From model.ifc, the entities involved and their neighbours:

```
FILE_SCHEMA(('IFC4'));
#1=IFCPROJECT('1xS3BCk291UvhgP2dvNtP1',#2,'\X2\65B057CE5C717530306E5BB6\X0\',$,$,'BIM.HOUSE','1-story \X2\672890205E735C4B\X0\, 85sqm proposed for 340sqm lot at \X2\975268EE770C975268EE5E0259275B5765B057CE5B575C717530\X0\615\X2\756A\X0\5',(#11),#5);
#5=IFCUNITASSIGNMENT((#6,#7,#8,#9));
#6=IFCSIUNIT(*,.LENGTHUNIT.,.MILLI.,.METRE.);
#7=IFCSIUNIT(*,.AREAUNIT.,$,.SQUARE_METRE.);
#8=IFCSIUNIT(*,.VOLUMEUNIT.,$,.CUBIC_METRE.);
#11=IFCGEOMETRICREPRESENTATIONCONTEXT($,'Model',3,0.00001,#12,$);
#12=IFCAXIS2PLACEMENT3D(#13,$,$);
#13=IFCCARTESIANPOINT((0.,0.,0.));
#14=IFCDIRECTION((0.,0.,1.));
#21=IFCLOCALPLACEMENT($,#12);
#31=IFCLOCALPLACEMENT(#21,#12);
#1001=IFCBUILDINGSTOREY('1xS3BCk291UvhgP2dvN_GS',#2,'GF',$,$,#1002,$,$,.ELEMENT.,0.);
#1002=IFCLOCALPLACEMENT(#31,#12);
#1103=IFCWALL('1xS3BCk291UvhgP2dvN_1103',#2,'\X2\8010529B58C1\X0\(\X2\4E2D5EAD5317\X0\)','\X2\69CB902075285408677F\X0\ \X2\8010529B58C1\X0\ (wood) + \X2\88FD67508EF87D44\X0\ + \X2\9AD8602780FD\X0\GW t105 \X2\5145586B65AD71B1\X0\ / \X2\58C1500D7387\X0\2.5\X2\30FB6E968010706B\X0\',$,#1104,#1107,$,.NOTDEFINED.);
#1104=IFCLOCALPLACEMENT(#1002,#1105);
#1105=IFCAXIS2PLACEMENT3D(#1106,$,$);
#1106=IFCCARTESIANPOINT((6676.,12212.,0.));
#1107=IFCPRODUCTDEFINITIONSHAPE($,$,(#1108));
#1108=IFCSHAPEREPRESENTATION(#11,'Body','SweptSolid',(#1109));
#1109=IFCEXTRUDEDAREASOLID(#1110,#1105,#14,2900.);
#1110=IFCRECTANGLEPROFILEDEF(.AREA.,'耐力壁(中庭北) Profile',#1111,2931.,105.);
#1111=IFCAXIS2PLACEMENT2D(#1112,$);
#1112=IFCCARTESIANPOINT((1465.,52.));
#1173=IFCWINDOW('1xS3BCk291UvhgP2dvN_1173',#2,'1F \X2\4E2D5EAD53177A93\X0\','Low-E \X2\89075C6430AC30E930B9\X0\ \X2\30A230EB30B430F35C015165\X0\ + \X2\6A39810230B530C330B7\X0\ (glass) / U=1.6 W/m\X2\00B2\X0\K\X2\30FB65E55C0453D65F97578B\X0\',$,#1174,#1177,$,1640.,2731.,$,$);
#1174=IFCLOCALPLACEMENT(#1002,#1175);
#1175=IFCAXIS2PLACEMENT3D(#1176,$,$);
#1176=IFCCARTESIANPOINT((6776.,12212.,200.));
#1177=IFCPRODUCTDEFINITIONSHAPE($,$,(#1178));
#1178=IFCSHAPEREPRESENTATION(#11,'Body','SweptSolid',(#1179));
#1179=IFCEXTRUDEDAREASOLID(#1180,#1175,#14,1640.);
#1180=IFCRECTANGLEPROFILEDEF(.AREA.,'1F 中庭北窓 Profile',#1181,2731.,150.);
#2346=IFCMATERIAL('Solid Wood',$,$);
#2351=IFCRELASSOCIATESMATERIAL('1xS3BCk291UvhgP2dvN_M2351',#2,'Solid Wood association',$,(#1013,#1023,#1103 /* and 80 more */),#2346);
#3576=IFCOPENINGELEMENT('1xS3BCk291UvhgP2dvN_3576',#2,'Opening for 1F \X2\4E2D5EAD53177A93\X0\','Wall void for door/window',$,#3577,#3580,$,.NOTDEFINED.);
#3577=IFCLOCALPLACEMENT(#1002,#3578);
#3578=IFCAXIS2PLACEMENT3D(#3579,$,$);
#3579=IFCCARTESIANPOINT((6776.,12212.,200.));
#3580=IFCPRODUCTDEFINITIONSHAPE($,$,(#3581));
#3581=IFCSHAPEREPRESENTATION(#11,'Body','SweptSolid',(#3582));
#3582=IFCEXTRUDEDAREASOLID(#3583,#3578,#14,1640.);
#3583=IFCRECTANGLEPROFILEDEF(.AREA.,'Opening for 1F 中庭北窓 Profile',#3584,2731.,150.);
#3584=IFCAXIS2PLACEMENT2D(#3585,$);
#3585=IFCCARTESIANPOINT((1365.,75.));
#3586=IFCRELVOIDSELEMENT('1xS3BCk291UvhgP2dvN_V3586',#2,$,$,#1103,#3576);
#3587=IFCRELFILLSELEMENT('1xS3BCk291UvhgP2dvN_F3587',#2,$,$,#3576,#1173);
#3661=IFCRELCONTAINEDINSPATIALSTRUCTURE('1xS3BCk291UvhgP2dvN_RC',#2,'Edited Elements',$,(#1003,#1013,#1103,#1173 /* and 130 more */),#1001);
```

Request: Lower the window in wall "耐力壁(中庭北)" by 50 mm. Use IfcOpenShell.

```python
import numpy as np
import ifcopenshell
import ifcopenshell.api.geometry
import ifcopenshell.util.placement
import ifcopenshell.util.unit

model = ifcopenshell.open("model.ifc")
unit_scale = ifcopenshell.util.unit.calculate_unit_scale(model)

window = model.by_id(1173)
opening = window.FillsVoids[0].RelatingOpeningElement
dz = -50.0

shift = np.array([0.0, 0.0, dz])
# The window is not placed relative to its opening, so move both.
for product in (opening, window):
    matrix = ifcopenshell.util.placement.get_local_placement(product.ObjectPlacement)
    matrix[:3, 3] += shift
    ifcopenshell.api.geometry.edit_object_placement(model, product=product, matrix=matrix, is_si=False)

print(f"moved by {dz * unit_scale:+.3f} m")

model.write("model-out.ifc")
```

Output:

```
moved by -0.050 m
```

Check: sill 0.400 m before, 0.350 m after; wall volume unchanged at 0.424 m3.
